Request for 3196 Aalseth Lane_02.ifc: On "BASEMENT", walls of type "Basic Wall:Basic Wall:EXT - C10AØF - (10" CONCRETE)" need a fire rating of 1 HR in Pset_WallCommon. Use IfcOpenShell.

First a look at what the model holds.

```python
import ifcopenshell
import ifcopenshell.util.element

model = ifcopenshell.open("3196 Aalseth Lane_02.ifc")
print(model.schema)
storey = next(s for s in model.by_type("IfcBuildingStorey") if s.Name == "BASEMENT")
walls = [e for e in ifcopenshell.util.element.get_decomposition(storey) if e.is_a("IfcWall")]
seen = {}
for e in walls:
    element_type = ifcopenshell.util.element.get_type(e)
    key = (element_type.Name if element_type != e and element_type else None, ifcopenshell.util.element.get_pset(e, "Pset_WallCommon", "FireRating"))
    seen[key] = seen.get(key, 0) + 1
for (name, value), count in sorted(seen.items(), key=str):
    print(count, "x", name, "|", value)
```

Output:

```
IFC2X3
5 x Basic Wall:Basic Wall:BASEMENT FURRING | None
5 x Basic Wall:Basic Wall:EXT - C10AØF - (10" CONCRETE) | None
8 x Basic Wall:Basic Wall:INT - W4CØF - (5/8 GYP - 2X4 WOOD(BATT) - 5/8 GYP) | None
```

```python
import ifcopenshell
import ifcopenshell.api.pset
import ifcopenshell.util.element

model = ifcopenshell.open("3196 Aalseth Lane_02.ifc")

storey = next(s for s in model.by_type("IfcBuildingStorey") if s.Name == "BASEMENT")
walls = [e for e in ifcopenshell.util.element.get_decomposition(storey) if e.is_a("IfcWall")]

count = 0
for e in walls:
    element_type = ifcopenshell.util.element.get_type(e)
    if element_type in (None, e) or element_type.Name != 'Basic Wall:Basic Wall:EXT - C10AØF - (10" CONCRETE)':
        continue
    # add_pset returns the element's existing set when there is one.
    pset = ifcopenshell.api.pset.add_pset(model, product=e, name="Pset_WallCommon")
    ifcopenshell.api.pset.edit_pset(model, pset=pset, properties={"FireRating": "1 HR"})
    count += 1

print(count, "walls updated")

model.write("3196 Aalseth Lane_02-out.ifc")
```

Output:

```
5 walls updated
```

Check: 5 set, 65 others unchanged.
